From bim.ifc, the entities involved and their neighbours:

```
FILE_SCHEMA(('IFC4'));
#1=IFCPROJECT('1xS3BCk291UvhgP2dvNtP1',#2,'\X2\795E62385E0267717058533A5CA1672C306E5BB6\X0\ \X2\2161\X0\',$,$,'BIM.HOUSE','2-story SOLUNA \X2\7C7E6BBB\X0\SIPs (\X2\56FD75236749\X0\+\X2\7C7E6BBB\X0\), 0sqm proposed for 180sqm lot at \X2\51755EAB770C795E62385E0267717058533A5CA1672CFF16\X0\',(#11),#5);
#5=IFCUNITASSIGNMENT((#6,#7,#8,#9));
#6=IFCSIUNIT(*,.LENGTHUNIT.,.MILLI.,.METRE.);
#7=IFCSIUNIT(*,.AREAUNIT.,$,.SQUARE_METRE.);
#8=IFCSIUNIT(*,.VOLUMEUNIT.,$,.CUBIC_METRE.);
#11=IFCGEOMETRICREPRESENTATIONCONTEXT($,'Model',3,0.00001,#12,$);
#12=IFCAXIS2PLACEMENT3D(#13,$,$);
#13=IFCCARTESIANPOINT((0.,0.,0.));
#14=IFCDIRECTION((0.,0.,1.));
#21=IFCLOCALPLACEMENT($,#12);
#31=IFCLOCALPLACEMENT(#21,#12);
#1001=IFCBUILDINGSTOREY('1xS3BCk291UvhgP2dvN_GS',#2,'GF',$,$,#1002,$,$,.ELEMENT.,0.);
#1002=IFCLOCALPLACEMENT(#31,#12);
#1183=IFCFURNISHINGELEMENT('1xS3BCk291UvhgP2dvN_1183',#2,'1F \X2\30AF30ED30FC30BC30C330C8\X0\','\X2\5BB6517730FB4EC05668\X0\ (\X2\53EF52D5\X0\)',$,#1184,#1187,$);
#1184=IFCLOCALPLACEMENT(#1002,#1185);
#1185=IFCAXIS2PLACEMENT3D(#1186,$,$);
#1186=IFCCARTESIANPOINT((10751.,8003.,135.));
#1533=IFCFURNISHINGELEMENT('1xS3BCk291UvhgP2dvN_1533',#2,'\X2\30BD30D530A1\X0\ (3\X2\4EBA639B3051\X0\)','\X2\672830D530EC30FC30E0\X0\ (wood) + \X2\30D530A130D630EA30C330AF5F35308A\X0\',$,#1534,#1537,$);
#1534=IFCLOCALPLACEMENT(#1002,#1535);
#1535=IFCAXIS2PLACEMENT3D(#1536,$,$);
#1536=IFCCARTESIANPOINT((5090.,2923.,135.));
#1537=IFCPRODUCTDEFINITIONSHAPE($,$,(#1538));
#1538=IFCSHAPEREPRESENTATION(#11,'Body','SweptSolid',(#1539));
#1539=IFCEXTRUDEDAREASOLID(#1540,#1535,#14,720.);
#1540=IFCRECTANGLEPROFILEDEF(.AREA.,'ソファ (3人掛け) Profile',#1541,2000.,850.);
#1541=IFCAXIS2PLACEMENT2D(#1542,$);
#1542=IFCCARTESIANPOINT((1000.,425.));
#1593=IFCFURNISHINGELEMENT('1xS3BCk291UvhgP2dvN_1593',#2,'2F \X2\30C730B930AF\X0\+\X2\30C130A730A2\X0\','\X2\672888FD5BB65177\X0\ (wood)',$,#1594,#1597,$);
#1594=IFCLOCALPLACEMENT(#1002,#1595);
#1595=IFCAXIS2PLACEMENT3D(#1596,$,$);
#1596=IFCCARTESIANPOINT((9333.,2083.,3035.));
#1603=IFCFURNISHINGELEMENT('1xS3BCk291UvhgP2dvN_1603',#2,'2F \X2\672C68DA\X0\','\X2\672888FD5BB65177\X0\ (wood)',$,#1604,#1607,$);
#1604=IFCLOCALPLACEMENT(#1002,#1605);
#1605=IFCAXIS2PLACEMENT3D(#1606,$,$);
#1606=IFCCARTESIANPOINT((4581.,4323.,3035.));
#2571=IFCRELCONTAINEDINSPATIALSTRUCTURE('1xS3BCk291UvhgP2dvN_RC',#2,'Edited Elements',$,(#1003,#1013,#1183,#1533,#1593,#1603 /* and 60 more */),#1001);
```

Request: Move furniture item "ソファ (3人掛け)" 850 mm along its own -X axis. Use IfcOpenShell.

```python
import ifcopenshell
import ifcopenshell.api.geometry
import ifcopenshell.util.placement

model = ifcopenshell.open("bim.ifc")

item = model.by_guid("1xS3BCk291UvhgP2dvN_1533")
matrix = ifcopenshell.util.placement.get_local_placement(item.ObjectPlacement)
matrix[:3, 3] -= matrix[:3, 0] * 850.0
ifcopenshell.api.geometry.edit_object_placement(model, product=item, matrix=matrix, is_si=False)

print(ifcopenshell.util.placement.get_local_placement(item.ObjectPlacement).round(3) + 0.0)

model.write("bim_updated.ifc")
```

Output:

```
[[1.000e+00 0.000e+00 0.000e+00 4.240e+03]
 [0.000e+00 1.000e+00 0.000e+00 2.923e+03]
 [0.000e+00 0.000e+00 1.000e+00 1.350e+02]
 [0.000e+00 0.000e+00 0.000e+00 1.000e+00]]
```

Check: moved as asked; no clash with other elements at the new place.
